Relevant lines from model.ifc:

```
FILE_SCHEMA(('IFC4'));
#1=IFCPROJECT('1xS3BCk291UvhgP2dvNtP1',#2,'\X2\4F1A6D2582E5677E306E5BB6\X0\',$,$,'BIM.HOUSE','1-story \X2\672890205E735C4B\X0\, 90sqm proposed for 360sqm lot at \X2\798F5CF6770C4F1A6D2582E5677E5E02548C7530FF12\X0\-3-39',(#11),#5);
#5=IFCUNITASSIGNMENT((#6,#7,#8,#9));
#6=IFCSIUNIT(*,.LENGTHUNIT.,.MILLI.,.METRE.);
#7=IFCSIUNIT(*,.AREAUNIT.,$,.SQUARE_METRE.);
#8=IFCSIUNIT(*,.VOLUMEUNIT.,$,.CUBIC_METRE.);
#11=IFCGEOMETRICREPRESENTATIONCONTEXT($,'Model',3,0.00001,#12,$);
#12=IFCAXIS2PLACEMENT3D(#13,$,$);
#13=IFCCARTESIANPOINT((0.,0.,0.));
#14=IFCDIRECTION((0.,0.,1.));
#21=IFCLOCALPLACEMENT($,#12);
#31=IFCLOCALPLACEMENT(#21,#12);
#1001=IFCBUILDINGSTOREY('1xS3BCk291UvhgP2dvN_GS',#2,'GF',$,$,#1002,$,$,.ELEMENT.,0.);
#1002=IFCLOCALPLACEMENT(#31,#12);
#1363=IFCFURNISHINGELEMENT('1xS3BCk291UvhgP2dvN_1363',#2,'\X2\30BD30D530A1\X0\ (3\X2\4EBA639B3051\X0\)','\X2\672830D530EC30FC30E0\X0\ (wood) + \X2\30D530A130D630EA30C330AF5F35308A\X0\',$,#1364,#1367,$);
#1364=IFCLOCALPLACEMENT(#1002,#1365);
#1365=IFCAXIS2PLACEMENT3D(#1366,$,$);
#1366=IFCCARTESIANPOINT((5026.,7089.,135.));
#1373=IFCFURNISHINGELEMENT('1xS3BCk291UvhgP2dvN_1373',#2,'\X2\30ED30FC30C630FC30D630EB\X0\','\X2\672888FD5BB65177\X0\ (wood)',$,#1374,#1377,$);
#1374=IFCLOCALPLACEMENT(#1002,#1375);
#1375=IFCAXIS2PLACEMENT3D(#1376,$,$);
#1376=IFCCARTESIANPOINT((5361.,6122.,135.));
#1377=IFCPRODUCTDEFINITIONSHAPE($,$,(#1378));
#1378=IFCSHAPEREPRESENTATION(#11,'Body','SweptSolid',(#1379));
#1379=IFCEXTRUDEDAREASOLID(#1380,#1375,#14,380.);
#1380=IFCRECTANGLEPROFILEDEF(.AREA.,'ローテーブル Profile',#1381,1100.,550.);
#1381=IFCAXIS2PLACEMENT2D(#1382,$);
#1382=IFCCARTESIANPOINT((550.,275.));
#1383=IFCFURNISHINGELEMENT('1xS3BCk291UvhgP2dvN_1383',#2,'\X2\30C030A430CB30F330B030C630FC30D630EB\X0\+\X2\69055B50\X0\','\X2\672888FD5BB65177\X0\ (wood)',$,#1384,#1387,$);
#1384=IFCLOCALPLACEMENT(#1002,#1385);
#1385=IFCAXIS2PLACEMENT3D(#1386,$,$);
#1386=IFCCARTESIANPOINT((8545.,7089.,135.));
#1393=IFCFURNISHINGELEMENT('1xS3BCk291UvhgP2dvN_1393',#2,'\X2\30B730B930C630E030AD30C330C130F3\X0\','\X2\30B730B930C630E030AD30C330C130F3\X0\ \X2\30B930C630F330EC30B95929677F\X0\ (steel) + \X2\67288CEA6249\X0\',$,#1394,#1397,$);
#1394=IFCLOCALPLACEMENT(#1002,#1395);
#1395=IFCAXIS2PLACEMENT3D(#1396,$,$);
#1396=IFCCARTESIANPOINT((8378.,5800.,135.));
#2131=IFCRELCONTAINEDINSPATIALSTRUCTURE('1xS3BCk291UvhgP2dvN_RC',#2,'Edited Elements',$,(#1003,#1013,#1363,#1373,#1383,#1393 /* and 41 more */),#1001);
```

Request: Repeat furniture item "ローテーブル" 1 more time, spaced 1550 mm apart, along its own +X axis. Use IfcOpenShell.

```python
import ifcopenshell
import ifcopenshell.api.geometry
import ifcopenshell.api.root
import ifcopenshell.util.element
import ifcopenshell.util.placement
import ifcopenshell.util.unit

model = ifcopenshell.open("model.ifc")
unit_scale = ifcopenshell.util.unit.calculate_unit_scale(model)


def reuse_history(source, copy):
    """copy_class also copies each property set's owner history, people and application; keep the originals."""
    for rel in copy.IsDefinedBy:
        if rel.is_a("IfcRelDefinesByProperties") and (history := rel.RelatingPropertyDefinition.OwnerHistory):
            rel.RelatingPropertyDefinition.OwnerHistory = source.OwnerHistory
            ifcopenshell.util.element.remove_deep2(model, history)


source = model.by_id(1373)
base = ifcopenshell.util.placement.get_local_placement(source.ObjectPlacement)
step = base[:3, 0] * 1.55 / unit_scale

for i in range(1, 2):
    copy = ifcopenshell.api.root.copy_class(model, product=source)
    copy.Representation = ifcopenshell.util.element.copy_deep(
        model, source.Representation, exclude=["IfcGeometricRepresentationContext", "IfcRepresentationMap"]
    )
    reuse_history(source, copy)
    matrix = base.copy()
    matrix[:3, 3] += i * step
    print("added at", matrix[:3, 3].round(3) + 0.0)
    ifcopenshell.api.geometry.edit_object_placement(model, product=copy, matrix=matrix, is_si=False)

model.write("model-out.ifc")
```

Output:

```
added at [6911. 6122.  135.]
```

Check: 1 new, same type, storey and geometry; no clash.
